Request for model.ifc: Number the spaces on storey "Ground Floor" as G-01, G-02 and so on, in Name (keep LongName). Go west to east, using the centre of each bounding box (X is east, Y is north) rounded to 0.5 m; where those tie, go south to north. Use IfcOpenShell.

First a look at what the model holds.

```python
import ifcopenshell
import ifcopenshell.util.element
import ifcopenshell.util.placement

model = ifcopenshell.open("model.ifc")
print(model.schema)
storey = next(s for s in model.by_type("IfcBuildingStorey") if s.Name == "Ground Floor")
spaces = [e for e in ifcopenshell.util.element.get_decomposition(storey) if e.is_a("IfcSpace")]
for e in sorted(spaces, key=lambda e: e.id()):
    origin = ifcopenshell.util.placement.get_local_placement(e.ObjectPlacement)[:3, 3]
    print(e.id(), e.Name, e.LongName, origin.round(2) + 0.0, sep=" | ")
```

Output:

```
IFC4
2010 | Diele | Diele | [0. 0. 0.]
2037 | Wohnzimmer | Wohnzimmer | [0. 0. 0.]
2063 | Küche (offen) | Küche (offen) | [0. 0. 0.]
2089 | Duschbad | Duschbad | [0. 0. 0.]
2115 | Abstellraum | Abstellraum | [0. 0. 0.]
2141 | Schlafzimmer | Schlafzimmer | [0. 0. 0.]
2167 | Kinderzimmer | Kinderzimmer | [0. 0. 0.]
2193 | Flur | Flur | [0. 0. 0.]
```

```python
import ifcopenshell
import ifcopenshell.geom
import ifcopenshell.util.element
import ifcopenshell.util.shape

model = ifcopenshell.open("model.ifc")
settings = ifcopenshell.geom.settings()
settings.set("use-world-coords", True)


def centre(element):
    shape = ifcopenshell.geom.create_shape(settings, element)
    return ifcopenshell.util.shape.get_bbox_centroid(shape.geometry)


storey = next(s for s in model.by_type("IfcBuildingStorey") if s.Name == "Ground Floor")
spaces = [e for e in ifcopenshell.util.element.get_decomposition(storey) if e.is_a("IfcSpace")]

# Insertion points can sit at a corner or the storey origin, so sort by the geometry (in metres).
centres = {e: centre(e) for e in spaces}
spaces.sort(key=lambda e: (round(centres[e][0] / 0.5), centres[e][1]))

for i, e in enumerate(spaces, start=1):
    number = f"G-{i:02d}"
    e.Name = number
    print(e.id(), number)

model.write("model-out.ifc")
```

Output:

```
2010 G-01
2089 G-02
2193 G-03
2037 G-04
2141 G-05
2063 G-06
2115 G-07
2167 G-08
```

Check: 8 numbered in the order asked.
